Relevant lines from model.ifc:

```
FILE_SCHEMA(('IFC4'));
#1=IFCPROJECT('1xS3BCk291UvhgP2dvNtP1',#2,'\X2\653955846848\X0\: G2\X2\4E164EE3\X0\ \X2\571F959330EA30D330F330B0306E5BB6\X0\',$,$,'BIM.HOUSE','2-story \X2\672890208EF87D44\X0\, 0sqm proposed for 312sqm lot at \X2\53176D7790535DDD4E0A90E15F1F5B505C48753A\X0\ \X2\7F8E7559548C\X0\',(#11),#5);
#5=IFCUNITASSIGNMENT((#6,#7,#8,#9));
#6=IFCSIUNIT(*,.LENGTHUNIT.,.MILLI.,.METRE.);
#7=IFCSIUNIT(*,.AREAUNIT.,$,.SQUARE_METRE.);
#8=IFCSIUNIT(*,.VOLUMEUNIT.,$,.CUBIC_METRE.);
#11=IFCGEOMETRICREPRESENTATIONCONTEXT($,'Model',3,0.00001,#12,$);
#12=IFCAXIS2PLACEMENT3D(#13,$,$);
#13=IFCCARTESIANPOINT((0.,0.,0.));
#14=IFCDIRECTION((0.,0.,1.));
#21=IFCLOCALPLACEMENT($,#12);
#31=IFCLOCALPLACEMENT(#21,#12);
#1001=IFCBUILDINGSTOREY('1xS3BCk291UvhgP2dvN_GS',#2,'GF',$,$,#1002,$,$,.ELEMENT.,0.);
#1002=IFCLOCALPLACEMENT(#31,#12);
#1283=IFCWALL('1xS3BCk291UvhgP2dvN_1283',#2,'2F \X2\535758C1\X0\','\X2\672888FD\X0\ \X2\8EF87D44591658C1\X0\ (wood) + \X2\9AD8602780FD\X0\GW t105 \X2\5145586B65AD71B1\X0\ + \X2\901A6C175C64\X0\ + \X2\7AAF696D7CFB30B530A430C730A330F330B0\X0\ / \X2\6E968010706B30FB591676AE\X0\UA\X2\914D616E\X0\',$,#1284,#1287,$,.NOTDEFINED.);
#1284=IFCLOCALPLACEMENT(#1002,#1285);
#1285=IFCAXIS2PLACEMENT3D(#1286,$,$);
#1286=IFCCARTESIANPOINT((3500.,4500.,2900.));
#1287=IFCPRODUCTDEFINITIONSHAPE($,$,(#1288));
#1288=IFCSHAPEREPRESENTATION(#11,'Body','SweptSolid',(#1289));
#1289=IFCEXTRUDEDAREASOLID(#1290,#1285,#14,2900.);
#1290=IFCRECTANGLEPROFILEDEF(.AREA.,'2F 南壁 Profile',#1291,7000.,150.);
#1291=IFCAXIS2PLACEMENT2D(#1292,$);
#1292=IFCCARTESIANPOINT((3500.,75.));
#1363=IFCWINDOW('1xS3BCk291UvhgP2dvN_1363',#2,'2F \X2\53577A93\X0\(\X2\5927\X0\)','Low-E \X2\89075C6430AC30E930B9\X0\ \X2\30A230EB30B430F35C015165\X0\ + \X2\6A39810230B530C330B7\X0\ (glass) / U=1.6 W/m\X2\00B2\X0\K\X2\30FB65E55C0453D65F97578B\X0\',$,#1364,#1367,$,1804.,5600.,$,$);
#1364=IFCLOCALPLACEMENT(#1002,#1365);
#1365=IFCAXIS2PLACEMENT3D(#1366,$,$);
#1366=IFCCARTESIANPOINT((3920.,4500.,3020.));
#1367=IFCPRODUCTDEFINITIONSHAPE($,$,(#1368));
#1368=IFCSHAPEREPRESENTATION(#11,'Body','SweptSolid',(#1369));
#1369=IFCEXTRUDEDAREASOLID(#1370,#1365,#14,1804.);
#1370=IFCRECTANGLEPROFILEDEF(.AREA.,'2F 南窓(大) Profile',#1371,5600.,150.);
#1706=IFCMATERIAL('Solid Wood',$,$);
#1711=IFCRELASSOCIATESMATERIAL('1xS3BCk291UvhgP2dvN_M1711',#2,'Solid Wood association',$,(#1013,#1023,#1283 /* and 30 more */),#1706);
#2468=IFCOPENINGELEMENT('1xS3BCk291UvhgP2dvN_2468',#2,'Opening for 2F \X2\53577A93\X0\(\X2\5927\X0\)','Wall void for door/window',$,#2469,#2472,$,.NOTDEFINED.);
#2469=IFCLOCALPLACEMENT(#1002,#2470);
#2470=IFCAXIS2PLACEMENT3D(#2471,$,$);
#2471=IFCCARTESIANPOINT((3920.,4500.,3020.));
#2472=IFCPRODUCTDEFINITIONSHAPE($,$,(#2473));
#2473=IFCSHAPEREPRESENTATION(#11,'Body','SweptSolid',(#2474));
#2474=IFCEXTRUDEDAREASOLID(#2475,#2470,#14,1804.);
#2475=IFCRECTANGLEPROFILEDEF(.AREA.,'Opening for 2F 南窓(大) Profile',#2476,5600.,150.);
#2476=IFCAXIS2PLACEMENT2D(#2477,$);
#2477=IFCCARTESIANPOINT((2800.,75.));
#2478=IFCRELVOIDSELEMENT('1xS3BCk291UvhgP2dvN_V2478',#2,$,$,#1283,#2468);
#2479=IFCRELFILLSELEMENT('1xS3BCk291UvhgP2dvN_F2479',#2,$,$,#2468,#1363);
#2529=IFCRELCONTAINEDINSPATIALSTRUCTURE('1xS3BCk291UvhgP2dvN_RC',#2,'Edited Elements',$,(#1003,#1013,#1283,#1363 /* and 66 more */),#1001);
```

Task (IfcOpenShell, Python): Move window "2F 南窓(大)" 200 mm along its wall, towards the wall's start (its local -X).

```python
import ifcopenshell
import ifcopenshell.api.geometry
import ifcopenshell.util.placement

model = ifcopenshell.open("model.ifc")

window = model.by_id(1363)
opening = window.FillsVoids[0].RelatingOpeningElement
wall = opening.VoidsElements[0].RelatingBuildingElement

wall_matrix = ifcopenshell.util.placement.get_local_placement(wall.ObjectPlacement)
shift = wall_matrix[:3, 0] * -200.0
before = ifcopenshell.util.placement.get_local_placement(window.ObjectPlacement)[:3, 3].copy()

# The window is not placed relative to its opening, so move both.
for product in (opening, window):
    matrix = ifcopenshell.util.placement.get_local_placement(product.ObjectPlacement)
    matrix[:3, 3] += shift
    ifcopenshell.api.geometry.edit_object_placement(model, product=product, matrix=matrix, is_si=False)

after = ifcopenshell.util.placement.get_local_placement(window.ObjectPlacement)[:3, 3]
print("window moved by", (after - before).round(3) + 0.0)

model.write("model_updated.ifc")
```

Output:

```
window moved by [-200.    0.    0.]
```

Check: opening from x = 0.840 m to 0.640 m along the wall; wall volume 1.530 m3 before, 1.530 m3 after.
